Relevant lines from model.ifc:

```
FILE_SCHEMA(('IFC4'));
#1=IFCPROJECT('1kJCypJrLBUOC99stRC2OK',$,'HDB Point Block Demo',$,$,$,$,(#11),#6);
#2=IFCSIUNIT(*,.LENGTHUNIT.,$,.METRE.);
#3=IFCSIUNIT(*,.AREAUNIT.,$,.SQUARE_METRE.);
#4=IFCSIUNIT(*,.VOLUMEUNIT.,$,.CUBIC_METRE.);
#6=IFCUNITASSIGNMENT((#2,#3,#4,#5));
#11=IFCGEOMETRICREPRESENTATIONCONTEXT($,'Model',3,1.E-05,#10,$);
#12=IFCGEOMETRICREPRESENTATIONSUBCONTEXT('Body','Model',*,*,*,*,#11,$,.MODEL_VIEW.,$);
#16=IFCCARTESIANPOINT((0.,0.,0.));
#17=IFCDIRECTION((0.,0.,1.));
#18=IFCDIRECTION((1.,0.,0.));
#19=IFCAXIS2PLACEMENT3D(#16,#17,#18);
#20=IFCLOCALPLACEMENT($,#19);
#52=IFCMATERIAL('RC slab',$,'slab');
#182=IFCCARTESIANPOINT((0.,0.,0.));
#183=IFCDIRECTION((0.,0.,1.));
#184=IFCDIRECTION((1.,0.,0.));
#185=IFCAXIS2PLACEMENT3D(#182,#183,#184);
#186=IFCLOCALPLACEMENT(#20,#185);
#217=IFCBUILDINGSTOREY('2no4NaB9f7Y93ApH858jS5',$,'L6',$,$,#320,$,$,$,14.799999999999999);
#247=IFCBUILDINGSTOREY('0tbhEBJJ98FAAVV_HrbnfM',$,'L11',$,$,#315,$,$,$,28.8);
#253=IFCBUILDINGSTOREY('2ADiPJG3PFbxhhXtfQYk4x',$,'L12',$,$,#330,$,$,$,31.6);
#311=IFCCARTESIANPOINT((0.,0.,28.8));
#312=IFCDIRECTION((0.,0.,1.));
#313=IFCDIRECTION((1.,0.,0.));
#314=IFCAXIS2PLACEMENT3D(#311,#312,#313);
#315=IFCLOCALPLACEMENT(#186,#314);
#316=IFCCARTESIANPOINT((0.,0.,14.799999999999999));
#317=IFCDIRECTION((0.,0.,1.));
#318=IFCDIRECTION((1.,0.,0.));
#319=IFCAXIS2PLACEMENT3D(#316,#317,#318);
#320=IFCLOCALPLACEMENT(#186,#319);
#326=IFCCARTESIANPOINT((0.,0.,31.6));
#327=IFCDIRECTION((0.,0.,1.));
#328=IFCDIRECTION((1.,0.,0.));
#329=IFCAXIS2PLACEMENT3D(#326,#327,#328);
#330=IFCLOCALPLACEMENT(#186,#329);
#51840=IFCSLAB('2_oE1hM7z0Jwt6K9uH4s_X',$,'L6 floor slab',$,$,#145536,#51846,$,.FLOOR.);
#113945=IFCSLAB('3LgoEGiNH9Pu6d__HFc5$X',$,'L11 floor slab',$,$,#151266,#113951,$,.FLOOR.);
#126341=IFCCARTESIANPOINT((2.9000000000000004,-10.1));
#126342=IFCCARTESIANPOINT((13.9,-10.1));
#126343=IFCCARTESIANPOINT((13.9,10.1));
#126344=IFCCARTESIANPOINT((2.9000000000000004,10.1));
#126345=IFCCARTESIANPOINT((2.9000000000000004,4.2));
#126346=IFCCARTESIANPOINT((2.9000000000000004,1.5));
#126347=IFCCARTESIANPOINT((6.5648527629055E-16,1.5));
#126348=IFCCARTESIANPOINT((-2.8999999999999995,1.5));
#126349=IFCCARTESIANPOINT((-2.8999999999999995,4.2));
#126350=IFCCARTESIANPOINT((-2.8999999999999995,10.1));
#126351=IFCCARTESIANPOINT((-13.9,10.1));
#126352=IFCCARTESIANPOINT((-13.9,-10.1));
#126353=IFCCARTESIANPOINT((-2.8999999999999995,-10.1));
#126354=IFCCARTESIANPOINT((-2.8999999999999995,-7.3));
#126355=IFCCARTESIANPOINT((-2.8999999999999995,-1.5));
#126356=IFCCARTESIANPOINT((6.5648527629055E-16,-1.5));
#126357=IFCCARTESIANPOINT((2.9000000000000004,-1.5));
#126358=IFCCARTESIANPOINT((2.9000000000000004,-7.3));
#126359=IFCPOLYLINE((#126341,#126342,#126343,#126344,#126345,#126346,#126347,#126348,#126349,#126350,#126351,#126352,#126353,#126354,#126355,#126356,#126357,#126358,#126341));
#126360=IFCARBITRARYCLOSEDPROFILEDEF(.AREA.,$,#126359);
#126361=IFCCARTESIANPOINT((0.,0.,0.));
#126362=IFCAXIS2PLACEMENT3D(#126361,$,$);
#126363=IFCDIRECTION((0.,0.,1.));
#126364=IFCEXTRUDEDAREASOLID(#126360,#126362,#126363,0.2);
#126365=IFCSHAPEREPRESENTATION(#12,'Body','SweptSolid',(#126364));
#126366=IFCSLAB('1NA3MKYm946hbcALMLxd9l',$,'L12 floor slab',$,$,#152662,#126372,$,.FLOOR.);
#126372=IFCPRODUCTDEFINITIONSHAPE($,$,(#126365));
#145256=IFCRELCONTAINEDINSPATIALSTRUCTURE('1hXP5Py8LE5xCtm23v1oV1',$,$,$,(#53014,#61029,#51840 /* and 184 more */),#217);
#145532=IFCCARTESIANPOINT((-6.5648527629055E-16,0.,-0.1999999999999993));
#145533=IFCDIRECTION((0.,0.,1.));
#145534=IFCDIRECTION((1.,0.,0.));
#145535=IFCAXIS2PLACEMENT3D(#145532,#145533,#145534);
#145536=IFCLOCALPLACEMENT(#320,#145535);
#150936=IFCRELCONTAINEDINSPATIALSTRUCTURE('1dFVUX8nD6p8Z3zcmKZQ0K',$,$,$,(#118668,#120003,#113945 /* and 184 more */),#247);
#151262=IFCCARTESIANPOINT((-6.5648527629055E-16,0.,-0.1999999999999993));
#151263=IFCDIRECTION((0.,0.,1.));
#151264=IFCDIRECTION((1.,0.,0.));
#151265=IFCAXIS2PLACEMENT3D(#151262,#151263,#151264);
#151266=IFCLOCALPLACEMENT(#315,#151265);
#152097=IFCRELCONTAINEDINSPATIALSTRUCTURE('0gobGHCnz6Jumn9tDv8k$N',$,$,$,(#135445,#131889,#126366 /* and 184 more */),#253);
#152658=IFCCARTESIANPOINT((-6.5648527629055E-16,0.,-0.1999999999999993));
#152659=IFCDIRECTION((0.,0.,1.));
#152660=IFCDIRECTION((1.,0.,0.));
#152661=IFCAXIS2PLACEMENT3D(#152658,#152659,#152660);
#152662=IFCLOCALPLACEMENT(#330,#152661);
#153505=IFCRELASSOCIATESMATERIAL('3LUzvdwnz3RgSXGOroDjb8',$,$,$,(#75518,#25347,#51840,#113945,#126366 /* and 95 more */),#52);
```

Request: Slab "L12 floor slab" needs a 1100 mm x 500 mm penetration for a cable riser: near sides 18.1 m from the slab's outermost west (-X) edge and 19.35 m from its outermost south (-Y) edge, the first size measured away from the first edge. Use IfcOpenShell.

```python
import numpy as np
import ifcopenshell
import ifcopenshell.api.feature
import ifcopenshell.api.geometry
import ifcopenshell.api.root
import ifcopenshell.geom
import ifcopenshell.util.placement
import ifcopenshell.util.representation
import ifcopenshell.util.shape
import ifcopenshell.util.unit

model = ifcopenshell.open("model.ifc")
unit_scale = ifcopenshell.util.unit.calculate_unit_scale(model)
settings = ifcopenshell.geom.settings()


def volume(element):
    """Net volume in cubic metres, openings subtracted."""
    shape = ifcopenshell.geom.create_shape(settings, element)
    return ifcopenshell.util.shape.get_volume(shape.geometry)


slab = model.by_guid("1NA3MKYm946hbcALMLxd9l")
before = volume(slab)

# Extent in the slab's own axes, in metres. The edges named are its -X and -Y sides.
slab_shape = ifcopenshell.geom.create_shape(settings, slab)
vertices = ifcopenshell.util.shape.get_vertices(slab_shape.geometry)
x_min, y_min, bottom = vertices.min(axis=0)
top = vertices[:, 2].max()

opening = ifcopenshell.api.root.create_entity(model, ifc_class="IfcOpeningElement", name="Cable riser opening", predefined_type="OPENING")
context = ifcopenshell.util.representation.get_context(model, "Model", "Body", "MODEL_VIEW")
width, depth = 1.1, 0.5
outline = [(0.0, 0.0), (width, 0.0), (width, depth), (0.0, depth), (0.0, 0.0)]
# Overshoot both faces by 50 mm so the cut is clean.
shape = ifcopenshell.api.geometry.add_slab_representation(
    model, context=context, depth=top - bottom + 0.1, polyline=outline
)
ifcopenshell.api.geometry.assign_representation(model, product=opening, representation=shape)

matrix = ifcopenshell.util.placement.get_local_placement(slab.ObjectPlacement)
matrix[:, 3] = matrix @ np.append(np.array([x_min + 18.1, y_min + 19.35, bottom - 0.05]) / unit_scale, 1.0)
ifcopenshell.api.geometry.edit_object_placement(model, product=opening, matrix=matrix, is_si=False)
ifcopenshell.api.feature.add_feature(model, feature=opening, element=slab)

after = volume(slab)

print(f"slab volume {before:.3f} -> {after:.3f} m3")

model.write("model_v2.ifc")
```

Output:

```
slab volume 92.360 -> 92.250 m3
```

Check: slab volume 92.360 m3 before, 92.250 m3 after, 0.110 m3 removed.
